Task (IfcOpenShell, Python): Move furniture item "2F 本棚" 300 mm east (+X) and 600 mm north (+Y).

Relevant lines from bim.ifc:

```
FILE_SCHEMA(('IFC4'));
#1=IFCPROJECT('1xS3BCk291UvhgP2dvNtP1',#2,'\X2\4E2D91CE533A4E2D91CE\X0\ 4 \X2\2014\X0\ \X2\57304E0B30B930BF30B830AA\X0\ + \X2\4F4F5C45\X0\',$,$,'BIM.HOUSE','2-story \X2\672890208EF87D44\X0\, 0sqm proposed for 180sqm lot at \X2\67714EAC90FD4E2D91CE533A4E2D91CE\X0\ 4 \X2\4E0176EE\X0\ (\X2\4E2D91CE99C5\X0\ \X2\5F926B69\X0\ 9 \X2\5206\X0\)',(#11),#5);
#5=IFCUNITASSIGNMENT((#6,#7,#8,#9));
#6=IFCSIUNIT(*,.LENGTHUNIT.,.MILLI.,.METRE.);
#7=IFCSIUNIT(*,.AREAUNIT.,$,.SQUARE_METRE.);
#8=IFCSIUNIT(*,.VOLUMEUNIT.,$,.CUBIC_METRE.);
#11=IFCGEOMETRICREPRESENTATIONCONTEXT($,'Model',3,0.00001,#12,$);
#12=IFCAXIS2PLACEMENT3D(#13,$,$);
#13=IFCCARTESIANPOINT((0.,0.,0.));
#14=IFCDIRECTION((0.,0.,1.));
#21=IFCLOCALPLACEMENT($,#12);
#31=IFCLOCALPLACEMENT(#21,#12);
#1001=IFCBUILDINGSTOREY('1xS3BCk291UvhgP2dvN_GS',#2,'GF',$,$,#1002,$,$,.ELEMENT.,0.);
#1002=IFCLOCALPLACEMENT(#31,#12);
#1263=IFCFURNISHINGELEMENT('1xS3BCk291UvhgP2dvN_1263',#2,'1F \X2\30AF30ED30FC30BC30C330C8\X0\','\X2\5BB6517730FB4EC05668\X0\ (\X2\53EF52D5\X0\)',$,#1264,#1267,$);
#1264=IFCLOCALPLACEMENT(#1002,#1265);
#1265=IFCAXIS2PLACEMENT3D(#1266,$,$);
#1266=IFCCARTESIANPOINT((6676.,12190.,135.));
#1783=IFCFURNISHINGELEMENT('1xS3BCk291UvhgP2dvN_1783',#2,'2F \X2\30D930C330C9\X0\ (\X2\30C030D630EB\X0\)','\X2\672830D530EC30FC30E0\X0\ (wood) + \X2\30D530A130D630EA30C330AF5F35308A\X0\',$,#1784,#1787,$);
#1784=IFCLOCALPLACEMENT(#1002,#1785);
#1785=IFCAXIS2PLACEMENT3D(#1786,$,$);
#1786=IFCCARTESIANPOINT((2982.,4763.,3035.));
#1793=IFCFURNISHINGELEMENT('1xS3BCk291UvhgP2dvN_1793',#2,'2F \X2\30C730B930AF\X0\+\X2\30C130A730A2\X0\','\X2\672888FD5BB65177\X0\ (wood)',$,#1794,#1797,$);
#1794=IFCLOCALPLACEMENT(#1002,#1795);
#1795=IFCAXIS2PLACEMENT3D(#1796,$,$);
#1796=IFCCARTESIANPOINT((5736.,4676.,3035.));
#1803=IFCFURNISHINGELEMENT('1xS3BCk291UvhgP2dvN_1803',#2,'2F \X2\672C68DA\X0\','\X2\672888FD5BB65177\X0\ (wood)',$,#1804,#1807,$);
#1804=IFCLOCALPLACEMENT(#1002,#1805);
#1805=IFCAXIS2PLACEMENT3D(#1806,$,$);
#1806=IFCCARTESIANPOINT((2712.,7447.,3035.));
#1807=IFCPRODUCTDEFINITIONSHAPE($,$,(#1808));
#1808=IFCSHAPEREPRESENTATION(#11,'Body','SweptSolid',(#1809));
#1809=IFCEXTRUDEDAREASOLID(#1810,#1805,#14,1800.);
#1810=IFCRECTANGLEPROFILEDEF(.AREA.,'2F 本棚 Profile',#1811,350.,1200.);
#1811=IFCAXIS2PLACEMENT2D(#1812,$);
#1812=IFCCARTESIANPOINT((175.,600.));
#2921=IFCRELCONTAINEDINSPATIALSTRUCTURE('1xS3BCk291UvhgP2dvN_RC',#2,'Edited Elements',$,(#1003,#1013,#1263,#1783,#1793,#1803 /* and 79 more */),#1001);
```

```python
import ifcopenshell
import ifcopenshell.api.geometry
import ifcopenshell.util.placement

model = ifcopenshell.open("bim.ifc")

item = model.by_id(1803)
matrix = ifcopenshell.util.placement.get_local_placement(item.ObjectPlacement)
matrix[0, 3] += 300.0
matrix[1, 3] += 600.0
ifcopenshell.api.geometry.edit_object_placement(model, product=item, matrix=matrix, is_si=False)

print(ifcopenshell.util.placement.get_local_placement(item.ObjectPlacement).round(3) + 0.0)

model.write("bim_rev.ifc")
```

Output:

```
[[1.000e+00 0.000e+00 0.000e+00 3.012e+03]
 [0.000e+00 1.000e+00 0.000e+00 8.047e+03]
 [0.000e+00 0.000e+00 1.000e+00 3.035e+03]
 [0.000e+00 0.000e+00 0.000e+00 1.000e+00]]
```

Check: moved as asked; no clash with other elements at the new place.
